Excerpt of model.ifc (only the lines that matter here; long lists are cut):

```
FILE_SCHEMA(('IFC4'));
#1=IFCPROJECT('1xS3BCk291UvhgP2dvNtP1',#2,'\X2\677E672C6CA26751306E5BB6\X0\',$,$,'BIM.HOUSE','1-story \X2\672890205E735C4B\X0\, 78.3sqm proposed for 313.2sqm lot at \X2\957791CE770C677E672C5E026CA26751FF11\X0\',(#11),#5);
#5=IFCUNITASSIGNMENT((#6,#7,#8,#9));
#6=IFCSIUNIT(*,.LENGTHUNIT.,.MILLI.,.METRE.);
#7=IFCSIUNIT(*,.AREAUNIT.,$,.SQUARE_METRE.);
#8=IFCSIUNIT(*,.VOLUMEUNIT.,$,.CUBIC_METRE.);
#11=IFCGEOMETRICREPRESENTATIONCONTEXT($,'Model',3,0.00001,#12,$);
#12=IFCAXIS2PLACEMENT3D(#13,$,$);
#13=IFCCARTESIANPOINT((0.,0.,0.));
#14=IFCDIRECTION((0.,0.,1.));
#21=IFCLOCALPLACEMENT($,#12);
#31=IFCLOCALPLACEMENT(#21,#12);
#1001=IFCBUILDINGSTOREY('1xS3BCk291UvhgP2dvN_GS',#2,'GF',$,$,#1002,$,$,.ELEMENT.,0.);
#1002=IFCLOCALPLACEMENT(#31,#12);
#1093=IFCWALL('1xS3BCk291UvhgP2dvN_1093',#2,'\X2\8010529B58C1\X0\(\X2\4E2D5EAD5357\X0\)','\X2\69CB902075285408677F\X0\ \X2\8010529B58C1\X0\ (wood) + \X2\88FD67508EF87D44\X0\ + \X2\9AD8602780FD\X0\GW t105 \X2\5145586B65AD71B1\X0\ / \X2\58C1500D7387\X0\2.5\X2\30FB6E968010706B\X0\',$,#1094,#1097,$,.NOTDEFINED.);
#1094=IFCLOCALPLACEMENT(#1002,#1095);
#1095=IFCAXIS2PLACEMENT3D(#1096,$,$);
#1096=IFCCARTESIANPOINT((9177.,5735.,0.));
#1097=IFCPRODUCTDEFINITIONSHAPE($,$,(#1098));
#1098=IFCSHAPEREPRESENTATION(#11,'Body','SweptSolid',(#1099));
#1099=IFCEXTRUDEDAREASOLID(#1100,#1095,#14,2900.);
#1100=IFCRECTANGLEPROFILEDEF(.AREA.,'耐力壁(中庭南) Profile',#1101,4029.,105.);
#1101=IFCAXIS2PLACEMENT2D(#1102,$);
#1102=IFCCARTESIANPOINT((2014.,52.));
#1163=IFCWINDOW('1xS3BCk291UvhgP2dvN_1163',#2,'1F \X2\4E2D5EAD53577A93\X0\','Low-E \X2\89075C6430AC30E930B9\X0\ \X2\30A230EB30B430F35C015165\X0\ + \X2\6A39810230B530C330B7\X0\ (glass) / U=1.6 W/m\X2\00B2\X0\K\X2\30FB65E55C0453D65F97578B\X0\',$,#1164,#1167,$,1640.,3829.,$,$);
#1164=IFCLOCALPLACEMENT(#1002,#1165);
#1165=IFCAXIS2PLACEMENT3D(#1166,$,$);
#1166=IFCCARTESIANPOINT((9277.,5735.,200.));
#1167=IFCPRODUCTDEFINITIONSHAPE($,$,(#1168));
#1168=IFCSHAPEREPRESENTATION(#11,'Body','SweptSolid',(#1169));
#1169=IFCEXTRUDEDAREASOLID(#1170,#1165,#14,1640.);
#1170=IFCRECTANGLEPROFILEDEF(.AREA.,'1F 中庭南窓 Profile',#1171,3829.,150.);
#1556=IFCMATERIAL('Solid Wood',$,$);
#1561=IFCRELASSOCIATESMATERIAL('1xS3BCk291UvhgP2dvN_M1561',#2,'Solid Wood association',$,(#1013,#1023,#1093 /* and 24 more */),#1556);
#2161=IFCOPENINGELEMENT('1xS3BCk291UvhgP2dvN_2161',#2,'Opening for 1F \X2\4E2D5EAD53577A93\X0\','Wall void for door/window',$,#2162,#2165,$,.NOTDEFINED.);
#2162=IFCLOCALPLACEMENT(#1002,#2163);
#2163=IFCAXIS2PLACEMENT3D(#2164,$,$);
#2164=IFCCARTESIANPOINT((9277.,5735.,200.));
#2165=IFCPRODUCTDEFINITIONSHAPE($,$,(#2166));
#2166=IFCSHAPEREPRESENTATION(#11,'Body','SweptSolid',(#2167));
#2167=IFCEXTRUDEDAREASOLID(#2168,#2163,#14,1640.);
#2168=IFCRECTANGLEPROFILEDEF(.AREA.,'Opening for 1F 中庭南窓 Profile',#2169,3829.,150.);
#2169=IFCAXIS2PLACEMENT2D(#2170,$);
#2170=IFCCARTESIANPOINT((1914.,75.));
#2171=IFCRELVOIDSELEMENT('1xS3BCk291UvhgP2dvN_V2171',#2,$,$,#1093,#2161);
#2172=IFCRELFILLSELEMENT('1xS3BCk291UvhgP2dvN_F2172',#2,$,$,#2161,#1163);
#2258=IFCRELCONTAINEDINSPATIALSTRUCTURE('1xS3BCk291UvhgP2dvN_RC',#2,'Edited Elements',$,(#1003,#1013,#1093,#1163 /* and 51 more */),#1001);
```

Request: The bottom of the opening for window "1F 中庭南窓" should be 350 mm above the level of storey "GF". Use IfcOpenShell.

```python
import numpy as np
import ifcopenshell
import ifcopenshell.api.geometry
import ifcopenshell.geom
import ifcopenshell.util.element
import ifcopenshell.util.placement
import ifcopenshell.util.shape
import ifcopenshell.util.unit

model = ifcopenshell.open("model.ifc")
unit_scale = ifcopenshell.util.unit.calculate_unit_scale(model)

window = model.by_guid("1xS3BCk291UvhgP2dvN_1163")
opening = window.FillsVoids[0].RelatingOpeningElement
storey = ifcopenshell.util.element.get_container(window, ifc_class="IfcBuildingStorey")
level = ifcopenshell.util.placement.get_local_placement(storey.ObjectPlacement)[2, 3]

# The opening's origin need not be at the sill, so measure its lowest point.
shape = ifcopenshell.geom.create_shape(ifcopenshell.geom.settings(), opening)
bottom = ifcopenshell.util.shape.get_shape_bottom_elevation(shape, shape.geometry) / unit_scale
dz = level + 350.0 - bottom

shift = np.array([0.0, 0.0, dz])
# The window is not placed relative to its opening, so move both.
for product in (opening, window):
    matrix = ifcopenshell.util.placement.get_local_placement(product.ObjectPlacement)
    matrix[:3, 3] += shift
    ifcopenshell.api.geometry.edit_object_placement(model, product=product, matrix=matrix, is_si=False)

print(f"moved by {dz * unit_scale:+.3f} m")

model.write("model_rev.ifc")
```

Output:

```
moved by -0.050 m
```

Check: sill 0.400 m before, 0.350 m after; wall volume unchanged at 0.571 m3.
